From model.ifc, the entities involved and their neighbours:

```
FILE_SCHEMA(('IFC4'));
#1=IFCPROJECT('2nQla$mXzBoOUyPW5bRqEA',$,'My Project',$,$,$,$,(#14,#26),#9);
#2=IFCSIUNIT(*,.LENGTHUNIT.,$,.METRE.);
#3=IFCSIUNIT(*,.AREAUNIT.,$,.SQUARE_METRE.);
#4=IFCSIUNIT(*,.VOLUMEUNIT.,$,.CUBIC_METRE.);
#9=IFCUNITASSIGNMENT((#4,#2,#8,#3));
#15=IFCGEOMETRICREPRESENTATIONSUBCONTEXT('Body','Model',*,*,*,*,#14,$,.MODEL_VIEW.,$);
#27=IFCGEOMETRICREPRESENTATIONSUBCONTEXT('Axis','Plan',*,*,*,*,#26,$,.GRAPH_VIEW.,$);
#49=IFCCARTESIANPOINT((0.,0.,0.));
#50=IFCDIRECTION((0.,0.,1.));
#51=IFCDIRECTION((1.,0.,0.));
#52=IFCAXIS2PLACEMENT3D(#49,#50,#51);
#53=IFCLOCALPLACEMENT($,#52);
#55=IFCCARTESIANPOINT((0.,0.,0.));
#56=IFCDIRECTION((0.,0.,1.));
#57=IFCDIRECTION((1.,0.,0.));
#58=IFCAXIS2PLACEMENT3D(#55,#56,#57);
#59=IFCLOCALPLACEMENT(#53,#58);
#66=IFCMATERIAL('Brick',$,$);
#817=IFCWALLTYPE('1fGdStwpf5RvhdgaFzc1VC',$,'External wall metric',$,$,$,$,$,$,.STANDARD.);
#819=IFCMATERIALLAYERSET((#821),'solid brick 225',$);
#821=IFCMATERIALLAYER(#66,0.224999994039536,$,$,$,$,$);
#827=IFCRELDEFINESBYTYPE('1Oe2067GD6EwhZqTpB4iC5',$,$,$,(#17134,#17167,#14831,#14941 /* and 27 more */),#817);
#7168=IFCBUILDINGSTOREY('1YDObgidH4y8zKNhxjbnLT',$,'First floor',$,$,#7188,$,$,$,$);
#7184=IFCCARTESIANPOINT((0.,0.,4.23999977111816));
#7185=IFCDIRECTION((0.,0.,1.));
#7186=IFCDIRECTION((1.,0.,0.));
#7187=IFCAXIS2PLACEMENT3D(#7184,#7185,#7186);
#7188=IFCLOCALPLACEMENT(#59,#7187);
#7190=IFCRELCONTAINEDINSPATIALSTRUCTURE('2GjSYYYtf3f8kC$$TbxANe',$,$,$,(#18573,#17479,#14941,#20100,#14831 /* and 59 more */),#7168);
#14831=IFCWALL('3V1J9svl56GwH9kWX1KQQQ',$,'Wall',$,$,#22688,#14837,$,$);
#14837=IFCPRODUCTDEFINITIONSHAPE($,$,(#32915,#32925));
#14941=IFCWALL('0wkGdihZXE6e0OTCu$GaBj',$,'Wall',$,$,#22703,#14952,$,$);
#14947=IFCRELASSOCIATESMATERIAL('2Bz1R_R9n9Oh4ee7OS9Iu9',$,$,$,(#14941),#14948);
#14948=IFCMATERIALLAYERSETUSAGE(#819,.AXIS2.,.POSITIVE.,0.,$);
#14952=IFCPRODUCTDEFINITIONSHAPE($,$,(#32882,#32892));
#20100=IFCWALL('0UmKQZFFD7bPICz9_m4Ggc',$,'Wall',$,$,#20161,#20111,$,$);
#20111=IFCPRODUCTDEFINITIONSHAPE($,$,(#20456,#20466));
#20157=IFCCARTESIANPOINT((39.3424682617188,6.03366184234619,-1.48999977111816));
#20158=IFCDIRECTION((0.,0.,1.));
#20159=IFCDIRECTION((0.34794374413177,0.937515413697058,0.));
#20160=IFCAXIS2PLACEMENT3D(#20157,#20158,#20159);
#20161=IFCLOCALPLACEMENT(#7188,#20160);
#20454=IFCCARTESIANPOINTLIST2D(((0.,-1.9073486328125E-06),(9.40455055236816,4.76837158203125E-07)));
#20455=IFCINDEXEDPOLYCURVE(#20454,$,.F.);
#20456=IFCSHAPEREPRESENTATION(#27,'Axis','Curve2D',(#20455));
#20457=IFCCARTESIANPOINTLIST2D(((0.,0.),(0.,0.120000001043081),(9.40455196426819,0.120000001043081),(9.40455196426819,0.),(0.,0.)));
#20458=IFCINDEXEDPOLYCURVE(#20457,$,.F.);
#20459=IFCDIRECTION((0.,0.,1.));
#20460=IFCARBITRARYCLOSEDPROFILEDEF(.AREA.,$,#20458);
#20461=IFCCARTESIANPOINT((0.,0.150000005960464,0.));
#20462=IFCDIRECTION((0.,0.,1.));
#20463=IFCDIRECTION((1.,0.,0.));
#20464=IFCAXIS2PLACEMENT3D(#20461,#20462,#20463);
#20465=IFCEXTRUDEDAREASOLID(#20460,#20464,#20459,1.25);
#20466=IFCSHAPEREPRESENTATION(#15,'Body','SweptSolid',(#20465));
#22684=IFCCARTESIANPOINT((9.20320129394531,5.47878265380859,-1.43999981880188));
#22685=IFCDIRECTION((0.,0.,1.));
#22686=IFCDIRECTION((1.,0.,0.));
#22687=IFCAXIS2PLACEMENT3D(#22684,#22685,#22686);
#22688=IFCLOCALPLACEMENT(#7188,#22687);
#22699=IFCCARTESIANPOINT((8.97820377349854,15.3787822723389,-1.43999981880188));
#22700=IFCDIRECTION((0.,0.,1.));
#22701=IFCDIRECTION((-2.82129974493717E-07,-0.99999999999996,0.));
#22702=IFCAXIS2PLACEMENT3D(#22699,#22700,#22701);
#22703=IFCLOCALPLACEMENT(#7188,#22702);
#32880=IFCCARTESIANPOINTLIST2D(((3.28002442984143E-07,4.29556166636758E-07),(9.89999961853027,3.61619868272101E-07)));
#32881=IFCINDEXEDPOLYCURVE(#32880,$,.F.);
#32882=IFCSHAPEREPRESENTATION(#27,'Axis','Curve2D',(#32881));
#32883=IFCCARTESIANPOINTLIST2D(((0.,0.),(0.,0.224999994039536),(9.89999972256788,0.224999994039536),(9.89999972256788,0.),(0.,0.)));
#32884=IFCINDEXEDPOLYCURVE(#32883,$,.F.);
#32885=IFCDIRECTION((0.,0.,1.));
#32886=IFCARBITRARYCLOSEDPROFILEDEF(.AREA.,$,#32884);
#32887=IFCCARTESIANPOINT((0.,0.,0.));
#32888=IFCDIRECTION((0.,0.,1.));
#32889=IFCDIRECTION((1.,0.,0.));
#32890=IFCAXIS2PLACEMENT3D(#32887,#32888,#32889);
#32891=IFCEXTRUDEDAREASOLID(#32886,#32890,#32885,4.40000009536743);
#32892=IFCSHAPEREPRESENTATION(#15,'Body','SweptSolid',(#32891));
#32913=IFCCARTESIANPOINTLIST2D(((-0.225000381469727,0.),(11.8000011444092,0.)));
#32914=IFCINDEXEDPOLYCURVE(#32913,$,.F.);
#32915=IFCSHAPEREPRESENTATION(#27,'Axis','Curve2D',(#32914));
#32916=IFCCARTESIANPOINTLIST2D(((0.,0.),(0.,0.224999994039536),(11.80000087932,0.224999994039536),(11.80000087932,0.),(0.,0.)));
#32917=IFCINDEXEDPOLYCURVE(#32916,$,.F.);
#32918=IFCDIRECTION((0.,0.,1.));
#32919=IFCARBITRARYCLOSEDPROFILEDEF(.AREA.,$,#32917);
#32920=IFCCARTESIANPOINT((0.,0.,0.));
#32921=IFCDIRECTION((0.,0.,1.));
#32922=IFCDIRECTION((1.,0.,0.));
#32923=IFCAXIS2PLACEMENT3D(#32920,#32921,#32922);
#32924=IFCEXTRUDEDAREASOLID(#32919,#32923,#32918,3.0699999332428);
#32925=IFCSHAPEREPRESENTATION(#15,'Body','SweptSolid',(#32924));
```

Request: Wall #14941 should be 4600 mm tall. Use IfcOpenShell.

```python
import ifcopenshell
import ifcopenshell.geom
import ifcopenshell.util.representation
import ifcopenshell.util.shape
import ifcopenshell.util.unit

model = ifcopenshell.open("model.ifc")
unit_scale = ifcopenshell.util.unit.calculate_unit_scale(model)
settings = ifcopenshell.geom.settings()


def volume(element):
    """Net volume in cubic metres, openings subtracted."""
    shape = ifcopenshell.geom.create_shape(settings, element)
    return ifcopenshell.util.shape.get_volume(shape.geometry)


wall = model.by_id(14941)
before = volume(wall)

body = ifcopenshell.util.representation.get_representation(wall, "Model", "Body")
solid = body.Items[0]
old_height = solid.Depth
solid.Depth = 4.6 / unit_scale
after = volume(wall)

print(f"height {old_height:g} -> {solid.Depth:g}, volume {before:.3f} -> {after:.3f} m3")

model.write("model_updated.ifc")
```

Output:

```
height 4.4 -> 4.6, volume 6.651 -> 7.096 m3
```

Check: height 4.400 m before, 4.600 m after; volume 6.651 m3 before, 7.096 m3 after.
